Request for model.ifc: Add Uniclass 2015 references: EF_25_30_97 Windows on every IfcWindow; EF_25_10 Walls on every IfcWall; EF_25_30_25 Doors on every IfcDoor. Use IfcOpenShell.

First a look at what the model holds.

```python
import ifcopenshell

model = ifcopenshell.open("model.ifc")
print(model.schema)
print("classifications:", [c.Name for c in model.by_type("IfcClassification")])
for ifc_class in ("IfcDoor", "IfcRoof", "IfcStair", "IfcWall", "IfcWindow"):
    print(ifc_class, len(model.by_type(ifc_class)))
```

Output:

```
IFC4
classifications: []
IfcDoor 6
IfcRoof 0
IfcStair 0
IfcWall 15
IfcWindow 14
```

```python
import ifcopenshell
import ifcopenshell.api.classification

model = ifcopenshell.open("model.ifc")

system = ifcopenshell.api.classification.add_classification(model, classification="Uniclass 2015")

codes = {
    "IfcWindow": ("EF_25_30_97", "Windows"),
    "IfcWall": ("EF_25_10", "Walls"),
    "IfcDoor": ("EF_25_30_25", "Doors"),
}
for ifc_class, (code, name) in codes.items():
    products = model.by_type(ifc_class)
    ifcopenshell.api.classification.add_reference(
        model, products=products, classification=system, identification=code, name=name
    )
    print(code, len(products))

model.write("model_edited.ifc")
```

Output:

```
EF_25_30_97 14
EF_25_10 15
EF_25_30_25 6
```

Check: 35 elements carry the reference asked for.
